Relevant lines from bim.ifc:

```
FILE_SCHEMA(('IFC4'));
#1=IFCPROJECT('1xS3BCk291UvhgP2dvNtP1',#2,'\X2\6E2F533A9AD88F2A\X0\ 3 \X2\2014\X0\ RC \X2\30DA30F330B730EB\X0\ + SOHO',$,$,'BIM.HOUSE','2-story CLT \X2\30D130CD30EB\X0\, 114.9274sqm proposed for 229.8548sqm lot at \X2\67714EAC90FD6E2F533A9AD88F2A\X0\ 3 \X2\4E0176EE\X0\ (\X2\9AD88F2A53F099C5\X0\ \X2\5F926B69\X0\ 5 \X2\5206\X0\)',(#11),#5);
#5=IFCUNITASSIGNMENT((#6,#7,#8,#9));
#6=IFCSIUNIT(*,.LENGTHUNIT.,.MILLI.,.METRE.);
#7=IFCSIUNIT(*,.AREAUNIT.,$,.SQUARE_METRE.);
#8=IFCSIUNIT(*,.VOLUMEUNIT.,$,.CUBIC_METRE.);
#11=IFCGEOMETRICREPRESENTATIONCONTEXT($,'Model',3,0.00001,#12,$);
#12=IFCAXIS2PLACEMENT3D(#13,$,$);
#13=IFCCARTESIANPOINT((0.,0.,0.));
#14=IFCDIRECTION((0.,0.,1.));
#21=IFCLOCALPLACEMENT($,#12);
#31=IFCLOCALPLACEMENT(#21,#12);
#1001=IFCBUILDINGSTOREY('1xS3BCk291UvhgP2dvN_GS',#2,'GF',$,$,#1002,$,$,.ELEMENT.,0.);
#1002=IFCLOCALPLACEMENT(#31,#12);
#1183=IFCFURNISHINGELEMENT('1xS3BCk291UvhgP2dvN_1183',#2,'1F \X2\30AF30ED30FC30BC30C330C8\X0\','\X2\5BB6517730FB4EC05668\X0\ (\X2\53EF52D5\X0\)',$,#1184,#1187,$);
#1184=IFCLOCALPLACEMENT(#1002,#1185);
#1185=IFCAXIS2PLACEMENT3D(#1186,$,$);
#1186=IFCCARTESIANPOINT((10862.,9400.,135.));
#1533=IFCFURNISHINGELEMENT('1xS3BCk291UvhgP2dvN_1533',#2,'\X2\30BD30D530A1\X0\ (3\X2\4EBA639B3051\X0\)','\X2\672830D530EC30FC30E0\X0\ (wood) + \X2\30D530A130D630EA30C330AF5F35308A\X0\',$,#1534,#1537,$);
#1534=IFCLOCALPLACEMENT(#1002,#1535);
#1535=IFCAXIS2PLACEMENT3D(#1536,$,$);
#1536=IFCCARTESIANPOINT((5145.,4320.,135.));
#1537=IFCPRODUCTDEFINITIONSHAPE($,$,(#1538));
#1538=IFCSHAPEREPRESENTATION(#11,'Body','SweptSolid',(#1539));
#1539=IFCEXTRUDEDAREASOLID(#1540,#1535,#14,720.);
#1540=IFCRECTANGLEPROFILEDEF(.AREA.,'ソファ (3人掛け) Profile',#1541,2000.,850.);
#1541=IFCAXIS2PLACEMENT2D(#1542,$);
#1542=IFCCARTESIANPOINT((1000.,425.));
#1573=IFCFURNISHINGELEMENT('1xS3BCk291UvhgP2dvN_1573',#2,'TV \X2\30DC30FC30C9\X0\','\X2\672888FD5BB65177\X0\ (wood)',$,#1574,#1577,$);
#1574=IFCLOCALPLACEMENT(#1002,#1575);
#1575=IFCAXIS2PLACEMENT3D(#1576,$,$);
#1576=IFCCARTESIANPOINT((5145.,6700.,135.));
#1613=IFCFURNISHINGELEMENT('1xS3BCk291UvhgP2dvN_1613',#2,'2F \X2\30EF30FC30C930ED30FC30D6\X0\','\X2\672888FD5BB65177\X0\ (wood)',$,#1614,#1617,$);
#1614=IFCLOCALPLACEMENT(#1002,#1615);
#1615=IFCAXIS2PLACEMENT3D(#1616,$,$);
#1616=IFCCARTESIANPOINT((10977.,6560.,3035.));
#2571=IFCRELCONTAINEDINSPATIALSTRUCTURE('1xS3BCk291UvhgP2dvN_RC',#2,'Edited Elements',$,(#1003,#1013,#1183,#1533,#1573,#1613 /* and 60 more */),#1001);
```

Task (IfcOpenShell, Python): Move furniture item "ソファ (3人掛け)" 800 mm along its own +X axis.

```python
import ifcopenshell
import ifcopenshell.api.geometry
import ifcopenshell.util.placement
import ifcopenshell.util.unit

model = ifcopenshell.open("bim.ifc")
unit_scale = ifcopenshell.util.unit.calculate_unit_scale(model)

item = model.by_guid("1xS3BCk291UvhgP2dvN_1533")
matrix = ifcopenshell.util.placement.get_local_placement(item.ObjectPlacement)
matrix[:3, 3] += matrix[:3, 0] * 0.8 / unit_scale
ifcopenshell.api.geometry.edit_object_placement(model, product=item, matrix=matrix, is_si=False)

print(ifcopenshell.util.placement.get_local_placement(item.ObjectPlacement).round(3) + 0.0)

model.write("bim_v2.ifc")
```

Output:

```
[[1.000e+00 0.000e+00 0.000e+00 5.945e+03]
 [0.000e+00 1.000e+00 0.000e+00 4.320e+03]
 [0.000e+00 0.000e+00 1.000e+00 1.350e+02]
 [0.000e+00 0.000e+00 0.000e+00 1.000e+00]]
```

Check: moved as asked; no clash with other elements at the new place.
